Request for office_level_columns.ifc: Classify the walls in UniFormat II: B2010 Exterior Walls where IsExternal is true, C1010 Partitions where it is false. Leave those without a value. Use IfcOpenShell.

First a look at what the model holds.

```python
import ifcopenshell
import ifcopenshell.util.element

model = ifcopenshell.open("office_level_columns.ifc")
print(model.schema)
print("classifications:", [c.Name for c in model.by_type("IfcClassification")])
values = [ifcopenshell.util.element.get_pset(e, "Pset_WallCommon", "IsExternal") for e in model.by_type("IfcWall")]
for value in (True, False, None):
    print("IsExternal", value, values.count(value))
```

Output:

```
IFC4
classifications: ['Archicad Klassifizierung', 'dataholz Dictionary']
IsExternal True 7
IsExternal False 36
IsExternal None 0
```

```python
import ifcopenshell
import ifcopenshell.api.classification
import ifcopenshell.util.element

model = ifcopenshell.open("office_level_columns.ifc")

system = ifcopenshell.api.classification.add_classification(model, classification="UniFormat II")

walls = model.by_type("IfcWall")
external = {e: ifcopenshell.util.element.get_pset(e, "Pset_WallCommon", "IsExternal") for e in walls}
for flag, code, name in ((True, "B2010", "Exterior Walls"), (False, "C1010", "Partitions")):
    products = [e for e in walls if external[e] is flag]
    ifcopenshell.api.classification.add_reference(
        model, products=products, classification=system, identification=code, name=name
    )
    print(code, len(products))

model.write("office_level_columns-out.ifc")
```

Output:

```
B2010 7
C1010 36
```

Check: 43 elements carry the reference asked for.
